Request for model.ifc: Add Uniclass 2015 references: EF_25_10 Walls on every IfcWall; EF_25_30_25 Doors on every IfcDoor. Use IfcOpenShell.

First a look at what the model holds.

```python
import ifcopenshell

model = ifcopenshell.open("model.ifc")
print(model.schema)
print("classifications:", [c.Name for c in model.by_type("IfcClassification")])
for ifc_class in ("IfcDoor", "IfcRoof", "IfcStair", "IfcWall", "IfcWindow"):
    print(ifc_class, len(model.by_type(ifc_class)))
```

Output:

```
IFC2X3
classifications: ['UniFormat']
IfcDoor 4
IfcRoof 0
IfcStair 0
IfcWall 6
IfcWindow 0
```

```python
import ifcopenshell
import ifcopenshell.api.classification

model = ifcopenshell.open("model.ifc")

# IFC2X3 requires Source and Edition and has no link from the project to the system.
system = model.create_entity("IfcClassification", Source="NBS", Edition="2015", Name="Uniclass 2015")

codes = {
    "IfcWall": ("EF_25_10", "Walls"),
    "IfcDoor": ("EF_25_30_25", "Doors"),
}
for ifc_class, (code, name) in codes.items():
    products = model.by_type(ifc_class)
    ifcopenshell.api.classification.add_reference(
        model, products=products, classification=system, identification=code, name=name
    )
    print(code, len(products))

model.write("model_edited.ifc")
```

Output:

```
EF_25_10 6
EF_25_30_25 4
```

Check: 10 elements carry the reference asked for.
